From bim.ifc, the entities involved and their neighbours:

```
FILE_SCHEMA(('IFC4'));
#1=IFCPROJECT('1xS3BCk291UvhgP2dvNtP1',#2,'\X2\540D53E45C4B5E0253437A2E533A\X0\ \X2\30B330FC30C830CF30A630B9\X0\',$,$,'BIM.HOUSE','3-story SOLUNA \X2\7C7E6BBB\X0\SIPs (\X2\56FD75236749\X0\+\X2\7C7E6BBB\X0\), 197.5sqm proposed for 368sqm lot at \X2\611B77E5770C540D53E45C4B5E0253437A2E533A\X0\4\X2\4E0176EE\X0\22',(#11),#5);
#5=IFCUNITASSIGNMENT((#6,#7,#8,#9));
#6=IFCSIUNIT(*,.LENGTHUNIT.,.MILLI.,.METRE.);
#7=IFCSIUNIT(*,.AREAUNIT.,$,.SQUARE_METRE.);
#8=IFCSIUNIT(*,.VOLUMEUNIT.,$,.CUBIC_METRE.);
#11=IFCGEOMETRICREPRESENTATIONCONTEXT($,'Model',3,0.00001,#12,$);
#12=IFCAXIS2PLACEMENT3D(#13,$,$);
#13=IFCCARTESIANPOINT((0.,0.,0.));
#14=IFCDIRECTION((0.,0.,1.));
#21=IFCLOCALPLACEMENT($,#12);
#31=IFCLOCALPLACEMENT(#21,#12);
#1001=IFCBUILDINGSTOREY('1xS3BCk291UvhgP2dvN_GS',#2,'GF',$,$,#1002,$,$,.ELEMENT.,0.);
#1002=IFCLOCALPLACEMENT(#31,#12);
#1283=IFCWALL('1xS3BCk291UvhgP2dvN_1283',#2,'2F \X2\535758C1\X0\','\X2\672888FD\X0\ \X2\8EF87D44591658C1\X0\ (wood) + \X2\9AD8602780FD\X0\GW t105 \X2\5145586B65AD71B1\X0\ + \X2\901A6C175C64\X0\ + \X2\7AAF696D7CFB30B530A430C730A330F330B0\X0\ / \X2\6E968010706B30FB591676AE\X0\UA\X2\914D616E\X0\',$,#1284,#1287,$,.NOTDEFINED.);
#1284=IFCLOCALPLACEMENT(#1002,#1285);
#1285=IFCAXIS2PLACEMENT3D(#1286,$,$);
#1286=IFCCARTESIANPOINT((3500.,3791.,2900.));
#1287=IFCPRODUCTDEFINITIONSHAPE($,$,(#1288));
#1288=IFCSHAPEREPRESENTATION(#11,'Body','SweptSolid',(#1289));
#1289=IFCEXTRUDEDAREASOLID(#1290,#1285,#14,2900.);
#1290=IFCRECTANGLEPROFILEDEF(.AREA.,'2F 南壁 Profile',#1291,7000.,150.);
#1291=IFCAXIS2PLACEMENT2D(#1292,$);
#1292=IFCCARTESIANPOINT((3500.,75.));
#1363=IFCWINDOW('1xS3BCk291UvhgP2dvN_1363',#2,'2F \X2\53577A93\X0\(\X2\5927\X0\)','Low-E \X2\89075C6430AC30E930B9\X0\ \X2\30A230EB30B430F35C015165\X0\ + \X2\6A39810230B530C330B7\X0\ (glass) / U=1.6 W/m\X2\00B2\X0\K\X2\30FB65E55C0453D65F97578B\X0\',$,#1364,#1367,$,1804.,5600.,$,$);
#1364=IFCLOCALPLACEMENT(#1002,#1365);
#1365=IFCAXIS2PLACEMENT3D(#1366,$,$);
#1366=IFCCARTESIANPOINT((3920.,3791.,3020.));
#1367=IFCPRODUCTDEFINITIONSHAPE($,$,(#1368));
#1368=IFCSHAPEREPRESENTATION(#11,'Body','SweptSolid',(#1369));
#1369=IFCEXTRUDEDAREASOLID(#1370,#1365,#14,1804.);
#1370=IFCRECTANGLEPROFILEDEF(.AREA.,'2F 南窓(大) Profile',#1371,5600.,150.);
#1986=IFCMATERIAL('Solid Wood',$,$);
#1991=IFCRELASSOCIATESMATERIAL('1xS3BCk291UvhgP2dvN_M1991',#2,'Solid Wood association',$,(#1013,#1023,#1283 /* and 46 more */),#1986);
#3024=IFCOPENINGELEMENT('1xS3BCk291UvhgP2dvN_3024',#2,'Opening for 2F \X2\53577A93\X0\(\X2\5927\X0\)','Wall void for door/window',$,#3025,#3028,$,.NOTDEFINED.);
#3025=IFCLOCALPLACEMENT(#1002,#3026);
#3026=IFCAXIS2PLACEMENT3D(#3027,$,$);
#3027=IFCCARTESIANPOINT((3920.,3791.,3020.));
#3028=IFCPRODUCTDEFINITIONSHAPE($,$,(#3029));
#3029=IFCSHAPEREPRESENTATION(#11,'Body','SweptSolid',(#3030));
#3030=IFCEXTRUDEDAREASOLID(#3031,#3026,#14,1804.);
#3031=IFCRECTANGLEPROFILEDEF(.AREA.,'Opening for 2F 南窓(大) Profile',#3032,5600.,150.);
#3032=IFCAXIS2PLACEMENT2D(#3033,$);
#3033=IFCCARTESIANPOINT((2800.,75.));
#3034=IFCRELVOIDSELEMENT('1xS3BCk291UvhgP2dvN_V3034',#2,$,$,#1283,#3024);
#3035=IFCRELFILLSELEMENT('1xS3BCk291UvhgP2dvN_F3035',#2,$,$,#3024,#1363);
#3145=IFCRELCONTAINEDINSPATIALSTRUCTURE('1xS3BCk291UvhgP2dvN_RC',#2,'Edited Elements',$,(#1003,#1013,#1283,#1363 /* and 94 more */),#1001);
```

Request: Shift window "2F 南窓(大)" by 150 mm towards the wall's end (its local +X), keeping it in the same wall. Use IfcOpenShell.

```python
import ifcopenshell
import ifcopenshell.api.geometry
import ifcopenshell.util.placement
import ifcopenshell.util.unit

model = ifcopenshell.open("bim.ifc")
unit_scale = ifcopenshell.util.unit.calculate_unit_scale(model)

window = model.by_id(1363)
opening = window.FillsVoids[0].RelatingOpeningElement
wall = opening.VoidsElements[0].RelatingBuildingElement

wall_matrix = ifcopenshell.util.placement.get_local_placement(wall.ObjectPlacement)
shift = wall_matrix[:3, 0] * 0.15 / unit_scale
before = ifcopenshell.util.placement.get_local_placement(window.ObjectPlacement)[:3, 3].copy()

# The window is not placed relative to its opening, so move both.
for product in (opening, window):
    matrix = ifcopenshell.util.placement.get_local_placement(product.ObjectPlacement)
    matrix[:3, 3] += shift
    ifcopenshell.api.geometry.edit_object_placement(model, product=product, matrix=matrix, is_si=False)

after = ifcopenshell.util.placement.get_local_placement(window.ObjectPlacement)[:3, 3]
print("window moved by", (after - before).round(3) + 0.0)

model.write("bim_v2.ifc")
```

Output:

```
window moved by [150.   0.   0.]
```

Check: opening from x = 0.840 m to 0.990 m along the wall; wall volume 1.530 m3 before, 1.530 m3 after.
